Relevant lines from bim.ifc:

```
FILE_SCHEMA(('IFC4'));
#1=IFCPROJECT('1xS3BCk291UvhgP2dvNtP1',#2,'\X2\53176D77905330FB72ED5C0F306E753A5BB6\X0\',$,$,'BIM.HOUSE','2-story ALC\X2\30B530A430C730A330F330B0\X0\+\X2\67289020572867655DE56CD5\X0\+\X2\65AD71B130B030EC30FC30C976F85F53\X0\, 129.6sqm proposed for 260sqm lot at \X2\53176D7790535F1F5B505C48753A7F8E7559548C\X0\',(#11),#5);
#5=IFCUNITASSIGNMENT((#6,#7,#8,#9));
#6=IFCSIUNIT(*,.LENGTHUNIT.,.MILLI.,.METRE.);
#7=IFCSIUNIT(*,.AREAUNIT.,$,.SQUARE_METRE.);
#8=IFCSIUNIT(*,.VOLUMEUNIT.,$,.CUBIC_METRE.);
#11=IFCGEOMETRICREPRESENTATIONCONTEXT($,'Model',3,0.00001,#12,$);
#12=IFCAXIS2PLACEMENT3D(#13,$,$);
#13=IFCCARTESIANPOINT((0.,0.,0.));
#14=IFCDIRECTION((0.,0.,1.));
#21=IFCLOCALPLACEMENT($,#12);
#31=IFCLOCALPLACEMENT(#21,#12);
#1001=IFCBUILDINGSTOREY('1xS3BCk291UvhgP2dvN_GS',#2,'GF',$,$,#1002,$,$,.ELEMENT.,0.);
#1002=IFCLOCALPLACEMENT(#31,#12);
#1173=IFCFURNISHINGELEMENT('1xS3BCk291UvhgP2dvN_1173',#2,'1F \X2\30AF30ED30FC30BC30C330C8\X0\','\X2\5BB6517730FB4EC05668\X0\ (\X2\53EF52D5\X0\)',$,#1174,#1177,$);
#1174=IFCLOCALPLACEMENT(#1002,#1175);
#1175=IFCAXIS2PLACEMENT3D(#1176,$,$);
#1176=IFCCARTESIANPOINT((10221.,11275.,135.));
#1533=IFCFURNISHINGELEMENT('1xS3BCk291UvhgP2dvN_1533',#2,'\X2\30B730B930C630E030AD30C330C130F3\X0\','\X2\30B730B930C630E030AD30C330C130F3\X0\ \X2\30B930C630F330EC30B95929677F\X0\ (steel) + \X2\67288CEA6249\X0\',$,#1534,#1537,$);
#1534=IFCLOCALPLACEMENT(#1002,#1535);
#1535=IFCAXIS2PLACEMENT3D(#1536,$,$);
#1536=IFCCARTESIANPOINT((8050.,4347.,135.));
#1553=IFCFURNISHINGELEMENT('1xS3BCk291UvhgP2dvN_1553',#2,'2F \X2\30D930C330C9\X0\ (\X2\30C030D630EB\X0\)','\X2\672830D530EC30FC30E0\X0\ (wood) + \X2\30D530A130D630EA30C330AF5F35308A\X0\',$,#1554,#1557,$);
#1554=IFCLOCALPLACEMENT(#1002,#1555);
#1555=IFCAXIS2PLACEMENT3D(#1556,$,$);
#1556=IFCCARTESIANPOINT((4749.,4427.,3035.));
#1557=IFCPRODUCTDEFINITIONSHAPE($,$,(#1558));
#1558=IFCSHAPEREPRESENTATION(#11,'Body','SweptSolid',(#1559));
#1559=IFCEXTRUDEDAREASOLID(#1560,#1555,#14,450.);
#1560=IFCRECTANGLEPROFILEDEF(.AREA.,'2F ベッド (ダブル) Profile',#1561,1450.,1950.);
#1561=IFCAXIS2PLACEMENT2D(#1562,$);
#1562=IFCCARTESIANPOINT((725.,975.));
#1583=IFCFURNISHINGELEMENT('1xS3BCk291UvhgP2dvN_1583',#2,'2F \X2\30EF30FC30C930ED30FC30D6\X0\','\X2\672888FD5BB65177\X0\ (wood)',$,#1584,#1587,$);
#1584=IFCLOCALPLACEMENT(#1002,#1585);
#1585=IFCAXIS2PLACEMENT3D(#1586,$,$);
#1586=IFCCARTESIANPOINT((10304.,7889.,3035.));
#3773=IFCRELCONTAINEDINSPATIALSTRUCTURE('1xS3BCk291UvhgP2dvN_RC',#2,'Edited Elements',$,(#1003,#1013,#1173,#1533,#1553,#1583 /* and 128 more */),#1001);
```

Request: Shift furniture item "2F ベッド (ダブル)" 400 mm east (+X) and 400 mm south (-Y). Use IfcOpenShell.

```python
import ifcopenshell
import ifcopenshell.api.geometry
import ifcopenshell.util.placement

model = ifcopenshell.open("bim.ifc")

item = model.by_guid("1xS3BCk291UvhgP2dvN_1553")
matrix = ifcopenshell.util.placement.get_local_placement(item.ObjectPlacement)
matrix[0, 3] += 400.0
matrix[1, 3] -= 400.0
ifcopenshell.api.geometry.edit_object_placement(model, product=item, matrix=matrix, is_si=False)

print(ifcopenshell.util.placement.get_local_placement(item.ObjectPlacement).round(3) + 0.0)

model.write("bim_updated.ifc")
```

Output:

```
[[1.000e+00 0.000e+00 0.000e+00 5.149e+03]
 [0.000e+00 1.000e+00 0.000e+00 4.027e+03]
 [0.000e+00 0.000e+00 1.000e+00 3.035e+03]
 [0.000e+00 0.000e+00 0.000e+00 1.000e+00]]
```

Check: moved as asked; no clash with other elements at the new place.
